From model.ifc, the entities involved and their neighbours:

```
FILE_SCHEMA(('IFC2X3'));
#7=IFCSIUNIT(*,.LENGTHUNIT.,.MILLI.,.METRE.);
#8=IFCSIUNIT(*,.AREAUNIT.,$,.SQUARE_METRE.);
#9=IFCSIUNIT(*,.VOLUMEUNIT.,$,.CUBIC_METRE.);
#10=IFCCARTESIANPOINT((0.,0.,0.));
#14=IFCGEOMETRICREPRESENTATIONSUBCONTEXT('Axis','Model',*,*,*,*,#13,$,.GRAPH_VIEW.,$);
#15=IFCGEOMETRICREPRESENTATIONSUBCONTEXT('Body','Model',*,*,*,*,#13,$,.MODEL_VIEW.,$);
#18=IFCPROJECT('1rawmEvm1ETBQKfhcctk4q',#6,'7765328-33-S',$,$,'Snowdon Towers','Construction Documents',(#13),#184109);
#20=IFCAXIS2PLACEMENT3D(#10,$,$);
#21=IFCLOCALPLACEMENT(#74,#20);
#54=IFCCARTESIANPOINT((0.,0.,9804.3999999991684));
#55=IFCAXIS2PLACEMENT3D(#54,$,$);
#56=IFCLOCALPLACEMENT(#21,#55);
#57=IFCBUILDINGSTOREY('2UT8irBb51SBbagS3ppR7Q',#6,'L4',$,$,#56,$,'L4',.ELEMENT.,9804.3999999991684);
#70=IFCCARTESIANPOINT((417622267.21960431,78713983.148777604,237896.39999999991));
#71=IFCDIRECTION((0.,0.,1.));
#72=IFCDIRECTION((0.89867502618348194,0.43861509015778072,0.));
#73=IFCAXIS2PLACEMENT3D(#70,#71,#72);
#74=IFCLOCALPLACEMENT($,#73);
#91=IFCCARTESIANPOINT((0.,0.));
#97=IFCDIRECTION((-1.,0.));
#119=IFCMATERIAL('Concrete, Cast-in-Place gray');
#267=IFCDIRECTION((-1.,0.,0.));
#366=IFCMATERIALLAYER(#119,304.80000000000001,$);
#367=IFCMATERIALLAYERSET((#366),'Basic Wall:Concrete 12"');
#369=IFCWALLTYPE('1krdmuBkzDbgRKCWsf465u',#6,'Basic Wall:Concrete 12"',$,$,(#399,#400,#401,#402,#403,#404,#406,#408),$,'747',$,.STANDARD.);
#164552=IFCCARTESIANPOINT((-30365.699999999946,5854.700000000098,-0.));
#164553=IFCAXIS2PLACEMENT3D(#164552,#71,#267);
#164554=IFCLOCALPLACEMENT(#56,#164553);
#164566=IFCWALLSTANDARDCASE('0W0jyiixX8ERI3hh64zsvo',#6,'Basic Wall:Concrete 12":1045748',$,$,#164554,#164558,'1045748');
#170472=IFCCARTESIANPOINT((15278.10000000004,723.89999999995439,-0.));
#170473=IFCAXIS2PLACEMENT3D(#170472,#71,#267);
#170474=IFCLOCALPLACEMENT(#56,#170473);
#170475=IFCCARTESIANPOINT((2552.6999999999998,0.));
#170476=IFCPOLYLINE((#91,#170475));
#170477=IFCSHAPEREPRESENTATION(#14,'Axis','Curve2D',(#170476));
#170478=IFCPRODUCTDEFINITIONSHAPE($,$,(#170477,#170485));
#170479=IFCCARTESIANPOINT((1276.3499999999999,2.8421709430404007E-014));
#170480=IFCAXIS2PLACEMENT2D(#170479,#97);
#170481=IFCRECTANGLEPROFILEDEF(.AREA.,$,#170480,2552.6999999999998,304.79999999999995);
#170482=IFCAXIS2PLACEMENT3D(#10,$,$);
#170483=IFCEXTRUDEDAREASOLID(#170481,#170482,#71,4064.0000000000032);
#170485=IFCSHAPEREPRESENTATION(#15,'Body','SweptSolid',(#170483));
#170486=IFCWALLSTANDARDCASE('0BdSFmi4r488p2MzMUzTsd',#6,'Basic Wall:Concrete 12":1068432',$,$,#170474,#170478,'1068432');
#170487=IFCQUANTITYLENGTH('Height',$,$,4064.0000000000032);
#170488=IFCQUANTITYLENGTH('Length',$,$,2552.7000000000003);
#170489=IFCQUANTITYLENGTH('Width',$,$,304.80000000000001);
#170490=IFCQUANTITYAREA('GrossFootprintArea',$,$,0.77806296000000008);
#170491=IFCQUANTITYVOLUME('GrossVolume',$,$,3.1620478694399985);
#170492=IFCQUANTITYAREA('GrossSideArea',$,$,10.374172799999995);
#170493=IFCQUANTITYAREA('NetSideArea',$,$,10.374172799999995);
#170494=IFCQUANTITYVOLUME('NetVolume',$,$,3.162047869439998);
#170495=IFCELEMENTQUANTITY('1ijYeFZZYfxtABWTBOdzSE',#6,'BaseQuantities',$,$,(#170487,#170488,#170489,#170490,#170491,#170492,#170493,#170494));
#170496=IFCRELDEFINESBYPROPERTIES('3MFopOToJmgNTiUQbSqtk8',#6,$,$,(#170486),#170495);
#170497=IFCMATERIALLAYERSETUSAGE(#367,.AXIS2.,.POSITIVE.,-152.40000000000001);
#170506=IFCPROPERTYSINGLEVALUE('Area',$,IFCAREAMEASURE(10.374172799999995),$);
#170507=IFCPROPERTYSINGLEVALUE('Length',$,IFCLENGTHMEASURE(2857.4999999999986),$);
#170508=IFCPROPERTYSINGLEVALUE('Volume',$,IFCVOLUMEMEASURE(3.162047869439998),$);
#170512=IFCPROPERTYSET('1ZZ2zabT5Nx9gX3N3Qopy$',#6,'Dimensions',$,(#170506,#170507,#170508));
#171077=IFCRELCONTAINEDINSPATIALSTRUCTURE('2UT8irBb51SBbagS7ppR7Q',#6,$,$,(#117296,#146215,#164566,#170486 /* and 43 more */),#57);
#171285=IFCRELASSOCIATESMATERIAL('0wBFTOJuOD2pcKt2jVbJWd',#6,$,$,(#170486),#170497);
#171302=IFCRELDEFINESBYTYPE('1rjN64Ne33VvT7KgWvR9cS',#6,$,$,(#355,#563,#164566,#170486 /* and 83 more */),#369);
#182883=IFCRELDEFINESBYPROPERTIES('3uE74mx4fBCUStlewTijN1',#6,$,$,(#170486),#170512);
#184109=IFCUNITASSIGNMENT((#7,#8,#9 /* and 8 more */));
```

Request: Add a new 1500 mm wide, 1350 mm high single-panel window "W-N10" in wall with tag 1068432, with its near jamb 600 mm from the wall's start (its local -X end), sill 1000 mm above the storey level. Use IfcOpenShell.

```python
import numpy as np
import ifcopenshell
import ifcopenshell.api.feature
import ifcopenshell.api.geometry
import ifcopenshell.api.pset
import ifcopenshell.api.root
import ifcopenshell.api.spatial
import ifcopenshell.api.type
import ifcopenshell.geom
import ifcopenshell.util.element
import ifcopenshell.util.placement
import ifcopenshell.util.representation
import ifcopenshell.util.shape
import ifcopenshell.util.unit

model = ifcopenshell.open("model.ifc")
unit_scale = ifcopenshell.util.unit.calculate_unit_scale(model)
area_scale = ifcopenshell.util.unit.calculate_unit_scale(model, "AREAUNIT")
volume_scale = ifcopenshell.util.unit.calculate_unit_scale(model, "VOLUMEUNIT")
settings = ifcopenshell.geom.settings()


def volume(element):
    """Net volume in cubic metres, openings subtracted."""
    shape = ifcopenshell.geom.create_shape(settings, element)
    return ifcopenshell.util.shape.get_volume(shape.geometry)


wall = model.by_id(170486)
storey = ifcopenshell.util.element.get_container(wall, ifc_class="IfcBuildingStorey")
context = ifcopenshell.util.representation.get_context(model, "Model", "Body", "MODEL_VIEW")
before = volume(wall)

width, height, from_end, sill = 1.5, 1.35, 0.6, 1  # metres

# The wall runs along its own X axis, and the end named is its -X end.
wall_shape = ifcopenshell.geom.create_shape(settings, wall)
x, y, z = ifcopenshell.util.shape.get_vertices(wall_shape.geometry).T
start = x.min() + from_end
face, thickness = float(y.min()), float(y.max() - y.min())
wall_matrix = ifcopenshell.util.placement.get_local_placement(wall.ObjectPlacement)
level = ifcopenshell.util.placement.get_local_placement(storey.ObjectPlacement)[2, 3]


def in_wall(x, y):
    """Placement at x, y metres in the wall's axes, at sill height."""
    matrix = wall_matrix.copy()
    matrix[:, 3] = wall_matrix @ np.array([x / unit_scale, y / unit_scale, 0.0, 1.0])
    matrix[2, 3] = level + sill / unit_scale
    return matrix


# Opening: a box that overshoots both wall faces by 50 mm.
opening = ifcopenshell.api.root.create_entity(model, ifc_class="IfcOpeningElement")
box = ifcopenshell.api.geometry.add_wall_representation(
    model, context=context, length=width, height=height, thickness=thickness + 0.1
)
ifcopenshell.api.geometry.assign_representation(model, product=opening, representation=box)
ifcopenshell.api.geometry.edit_object_placement(model, product=opening, matrix=in_wall(start, face - 0.05), is_si=False)
ifcopenshell.api.feature.add_feature(model, feature=opening, element=wall)

window = ifcopenshell.api.root.create_entity(model, ifc_class="IfcWindow", name="W-N10")
window.OverallWidth, window.OverallHeight = width / unit_scale, height / unit_scale
body = ifcopenshell.api.geometry.add_window_representation(
    model,
    context=context,
    overall_width=window.OverallWidth,
    overall_height=window.OverallHeight,
    partition_type="SINGLE_PANEL",
)
ifcopenshell.api.geometry.assign_representation(model, product=window, representation=body)
ifcopenshell.api.spatial.assign_container(model, products=[window], relating_structure=storey)
fills = ifcopenshell.api.feature.add_filling(model, opening=opening, element=window)
fills.OwnerHistory = window.OwnerHistory  # required in IFC2X3

# IFC2X3 keeps the operation on the window style.
style = ifcopenshell.api.root.create_entity(model, ifc_class="IfcWindowStyle", name="W-N10")
style.OperationType, style.ConstructionType = "SINGLE_PANEL", "NOTDEFINED"
style.ParameterTakesPrecedence = style.Sizeable = False
ifcopenshell.api.type.assign_type(model, related_objects=[window], relating_type=style)

# Centre the window in the wall's thickness.
ifcopenshell.api.geometry.edit_object_placement(model, product=window, matrix=in_wall(start, face), is_si=False)
window_shape = ifcopenshell.geom.create_shape(settings, window)
depth = ifcopenshell.util.shape.get_vertices(window_shape.geometry)[:, 1]
offset = face + thickness / 2 - (depth.min() + depth.max()) / 2
ifcopenshell.api.geometry.edit_object_placement(model, product=window, matrix=in_wall(start, offset), is_si=False)

after = volume(wall)

# Update the wall's stored quantities.
qto = model.by_id(ifcopenshell.util.element.get_pset(wall, "BaseQuantities", should_inherit=False)["id"])
ifcopenshell.api.pset.edit_qto(model, qto=qto, properties={
    "NetSideArea": after / thickness / area_scale,
    "NetVolume": after / volume_scale,
})
pset = model.by_id(ifcopenshell.util.element.get_pset(wall, "Dimensions", should_inherit=False)["id"])
ifcopenshell.api.pset.edit_pset(model, pset=pset, properties={
    "Area": model.create_entity("IfcAreaMeasure", after / thickness / area_scale),
    "Volume": model.create_entity("IfcVolumeMeasure", after / volume_scale),
})

print(f"wall volume {before:.3f} -> {after:.3f} m3")

model.write("model_rev.ifc")
```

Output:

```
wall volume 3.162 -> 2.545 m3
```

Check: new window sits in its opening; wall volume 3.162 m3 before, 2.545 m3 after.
